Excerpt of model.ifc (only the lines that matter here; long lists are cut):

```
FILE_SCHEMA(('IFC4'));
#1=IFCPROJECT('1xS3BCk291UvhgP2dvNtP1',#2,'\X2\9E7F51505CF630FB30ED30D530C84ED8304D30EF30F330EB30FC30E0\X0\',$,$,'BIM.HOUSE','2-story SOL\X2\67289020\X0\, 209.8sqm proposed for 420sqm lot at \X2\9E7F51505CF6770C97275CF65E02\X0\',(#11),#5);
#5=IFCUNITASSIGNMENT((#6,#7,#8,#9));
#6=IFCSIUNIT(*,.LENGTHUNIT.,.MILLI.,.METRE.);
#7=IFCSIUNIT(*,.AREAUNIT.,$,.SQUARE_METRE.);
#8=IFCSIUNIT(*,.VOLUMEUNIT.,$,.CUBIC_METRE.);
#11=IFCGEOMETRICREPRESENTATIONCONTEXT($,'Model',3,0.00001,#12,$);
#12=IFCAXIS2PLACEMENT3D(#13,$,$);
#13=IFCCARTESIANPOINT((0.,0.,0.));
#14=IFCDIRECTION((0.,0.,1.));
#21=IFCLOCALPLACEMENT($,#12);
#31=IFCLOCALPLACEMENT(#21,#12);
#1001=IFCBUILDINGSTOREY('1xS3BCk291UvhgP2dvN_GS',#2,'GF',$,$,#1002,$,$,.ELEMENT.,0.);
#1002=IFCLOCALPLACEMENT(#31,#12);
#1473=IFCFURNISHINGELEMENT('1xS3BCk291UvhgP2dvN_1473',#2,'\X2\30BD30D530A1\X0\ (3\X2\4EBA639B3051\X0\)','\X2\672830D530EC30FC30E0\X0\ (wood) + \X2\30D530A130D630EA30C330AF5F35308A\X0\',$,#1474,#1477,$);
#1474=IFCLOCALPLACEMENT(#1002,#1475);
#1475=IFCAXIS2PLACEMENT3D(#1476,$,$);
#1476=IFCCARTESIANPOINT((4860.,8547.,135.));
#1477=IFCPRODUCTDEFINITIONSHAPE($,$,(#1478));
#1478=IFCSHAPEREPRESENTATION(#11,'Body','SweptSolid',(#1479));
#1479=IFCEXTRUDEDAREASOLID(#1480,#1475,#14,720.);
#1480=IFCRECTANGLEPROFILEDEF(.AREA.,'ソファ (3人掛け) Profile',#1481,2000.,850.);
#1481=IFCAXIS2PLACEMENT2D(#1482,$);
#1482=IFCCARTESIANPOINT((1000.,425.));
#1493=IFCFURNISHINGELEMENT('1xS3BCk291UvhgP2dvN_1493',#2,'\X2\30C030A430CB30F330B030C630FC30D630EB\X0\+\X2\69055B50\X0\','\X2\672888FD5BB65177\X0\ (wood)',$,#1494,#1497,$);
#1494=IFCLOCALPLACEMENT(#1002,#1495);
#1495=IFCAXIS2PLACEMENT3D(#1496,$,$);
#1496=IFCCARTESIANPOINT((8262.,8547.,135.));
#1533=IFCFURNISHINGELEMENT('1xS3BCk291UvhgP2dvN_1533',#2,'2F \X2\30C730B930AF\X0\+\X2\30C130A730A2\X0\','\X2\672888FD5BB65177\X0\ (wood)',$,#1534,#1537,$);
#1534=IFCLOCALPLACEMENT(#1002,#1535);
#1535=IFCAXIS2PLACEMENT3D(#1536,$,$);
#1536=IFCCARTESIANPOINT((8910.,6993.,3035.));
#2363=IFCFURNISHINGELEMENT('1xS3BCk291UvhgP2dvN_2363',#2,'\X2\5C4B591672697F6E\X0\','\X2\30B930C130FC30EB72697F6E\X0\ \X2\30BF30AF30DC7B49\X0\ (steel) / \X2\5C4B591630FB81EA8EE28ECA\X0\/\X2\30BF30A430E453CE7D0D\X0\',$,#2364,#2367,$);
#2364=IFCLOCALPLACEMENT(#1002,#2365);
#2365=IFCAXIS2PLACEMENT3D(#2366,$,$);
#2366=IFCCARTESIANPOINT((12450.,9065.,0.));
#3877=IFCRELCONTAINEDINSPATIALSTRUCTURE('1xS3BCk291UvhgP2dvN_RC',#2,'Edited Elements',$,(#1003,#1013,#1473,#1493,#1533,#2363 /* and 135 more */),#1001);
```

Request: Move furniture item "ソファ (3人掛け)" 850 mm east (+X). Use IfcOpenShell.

```python
import ifcopenshell
import ifcopenshell.api.geometry
import ifcopenshell.util.placement
import ifcopenshell.util.unit

model = ifcopenshell.open("model.ifc")
unit_scale = ifcopenshell.util.unit.calculate_unit_scale(model)

item = model.by_guid("1xS3BCk291UvhgP2dvN_1473")
matrix = ifcopenshell.util.placement.get_local_placement(item.ObjectPlacement)
matrix[0, 3] += 0.85 / unit_scale
ifcopenshell.api.geometry.edit_object_placement(model, product=item, matrix=matrix, is_si=False)

print(ifcopenshell.util.placement.get_local_placement(item.ObjectPlacement).round(3) + 0.0)

model.write("model_v2.ifc")
```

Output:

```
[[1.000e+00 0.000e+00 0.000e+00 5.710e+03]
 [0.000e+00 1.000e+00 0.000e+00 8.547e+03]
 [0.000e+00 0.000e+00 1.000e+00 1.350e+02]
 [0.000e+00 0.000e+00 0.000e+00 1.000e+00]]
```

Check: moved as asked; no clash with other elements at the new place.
